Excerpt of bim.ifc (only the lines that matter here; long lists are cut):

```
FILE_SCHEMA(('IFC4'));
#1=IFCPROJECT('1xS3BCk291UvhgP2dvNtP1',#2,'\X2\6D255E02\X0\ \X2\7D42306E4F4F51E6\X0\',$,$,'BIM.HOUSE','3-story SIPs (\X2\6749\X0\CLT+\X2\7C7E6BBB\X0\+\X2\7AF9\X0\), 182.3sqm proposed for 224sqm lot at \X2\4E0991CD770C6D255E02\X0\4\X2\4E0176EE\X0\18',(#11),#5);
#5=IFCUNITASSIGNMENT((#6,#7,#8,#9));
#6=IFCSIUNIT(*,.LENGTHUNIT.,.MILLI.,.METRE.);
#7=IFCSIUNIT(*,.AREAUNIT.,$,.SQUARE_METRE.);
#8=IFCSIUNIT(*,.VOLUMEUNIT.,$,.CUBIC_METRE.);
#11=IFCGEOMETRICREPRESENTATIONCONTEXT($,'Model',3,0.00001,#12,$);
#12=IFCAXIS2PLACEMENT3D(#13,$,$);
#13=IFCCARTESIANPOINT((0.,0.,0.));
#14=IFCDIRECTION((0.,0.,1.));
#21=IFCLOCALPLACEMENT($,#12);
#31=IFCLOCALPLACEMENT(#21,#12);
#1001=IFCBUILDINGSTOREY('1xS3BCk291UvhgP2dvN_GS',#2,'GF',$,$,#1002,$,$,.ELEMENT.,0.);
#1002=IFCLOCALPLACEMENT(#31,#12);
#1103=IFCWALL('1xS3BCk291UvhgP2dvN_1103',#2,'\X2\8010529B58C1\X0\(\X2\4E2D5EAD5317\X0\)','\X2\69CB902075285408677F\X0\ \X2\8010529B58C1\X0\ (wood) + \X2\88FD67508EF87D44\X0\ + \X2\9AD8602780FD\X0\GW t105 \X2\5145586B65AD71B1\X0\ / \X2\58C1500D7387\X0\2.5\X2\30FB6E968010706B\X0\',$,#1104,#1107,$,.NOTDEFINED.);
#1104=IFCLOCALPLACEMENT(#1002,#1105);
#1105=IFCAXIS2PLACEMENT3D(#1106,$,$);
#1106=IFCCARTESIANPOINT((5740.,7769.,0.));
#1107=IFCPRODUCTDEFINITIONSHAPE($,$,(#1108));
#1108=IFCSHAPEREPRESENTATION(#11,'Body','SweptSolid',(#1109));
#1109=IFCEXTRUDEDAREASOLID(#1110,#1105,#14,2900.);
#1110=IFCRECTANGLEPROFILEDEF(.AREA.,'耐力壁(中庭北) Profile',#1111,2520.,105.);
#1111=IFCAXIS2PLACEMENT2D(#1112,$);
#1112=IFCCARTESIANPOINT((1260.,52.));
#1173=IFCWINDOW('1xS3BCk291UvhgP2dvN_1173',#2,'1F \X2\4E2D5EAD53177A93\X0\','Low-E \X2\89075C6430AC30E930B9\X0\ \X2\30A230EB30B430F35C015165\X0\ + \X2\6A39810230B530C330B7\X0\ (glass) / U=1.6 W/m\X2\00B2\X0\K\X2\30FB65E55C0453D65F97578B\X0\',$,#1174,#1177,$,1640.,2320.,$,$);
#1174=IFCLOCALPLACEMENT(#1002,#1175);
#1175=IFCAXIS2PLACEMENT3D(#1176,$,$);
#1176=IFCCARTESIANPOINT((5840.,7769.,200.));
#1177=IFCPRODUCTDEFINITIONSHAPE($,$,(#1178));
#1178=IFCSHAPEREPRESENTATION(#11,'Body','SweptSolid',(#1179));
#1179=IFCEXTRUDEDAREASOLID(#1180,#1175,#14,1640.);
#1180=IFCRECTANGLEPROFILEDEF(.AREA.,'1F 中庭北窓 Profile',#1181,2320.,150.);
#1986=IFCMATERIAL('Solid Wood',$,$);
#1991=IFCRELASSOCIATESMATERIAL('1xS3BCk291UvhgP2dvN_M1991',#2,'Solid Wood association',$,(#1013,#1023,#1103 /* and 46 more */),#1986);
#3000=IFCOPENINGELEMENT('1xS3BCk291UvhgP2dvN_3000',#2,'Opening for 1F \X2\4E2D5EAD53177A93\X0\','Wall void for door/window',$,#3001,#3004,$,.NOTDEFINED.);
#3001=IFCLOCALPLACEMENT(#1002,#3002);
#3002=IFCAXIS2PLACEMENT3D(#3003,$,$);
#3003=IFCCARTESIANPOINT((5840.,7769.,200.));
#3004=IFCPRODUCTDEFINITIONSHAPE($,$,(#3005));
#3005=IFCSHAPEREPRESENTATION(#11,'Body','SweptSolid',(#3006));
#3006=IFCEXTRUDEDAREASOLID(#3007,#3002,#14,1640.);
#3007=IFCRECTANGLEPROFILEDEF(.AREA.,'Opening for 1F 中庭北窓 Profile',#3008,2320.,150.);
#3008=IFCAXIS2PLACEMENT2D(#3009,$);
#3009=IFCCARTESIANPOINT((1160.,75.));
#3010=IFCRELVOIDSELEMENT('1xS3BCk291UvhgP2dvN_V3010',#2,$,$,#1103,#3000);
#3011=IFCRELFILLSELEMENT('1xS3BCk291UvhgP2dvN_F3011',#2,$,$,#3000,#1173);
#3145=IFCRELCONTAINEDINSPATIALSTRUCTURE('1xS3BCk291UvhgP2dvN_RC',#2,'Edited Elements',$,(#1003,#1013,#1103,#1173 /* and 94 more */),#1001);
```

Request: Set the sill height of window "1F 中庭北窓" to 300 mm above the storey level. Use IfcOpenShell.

```python
import numpy as np
import ifcopenshell
import ifcopenshell.api.geometry
import ifcopenshell.geom
import ifcopenshell.util.element
import ifcopenshell.util.placement
import ifcopenshell.util.shape
import ifcopenshell.util.unit

model = ifcopenshell.open("bim.ifc")
unit_scale = ifcopenshell.util.unit.calculate_unit_scale(model)

window = model.by_guid("1xS3BCk291UvhgP2dvN_1173")
opening = window.FillsVoids[0].RelatingOpeningElement
storey = ifcopenshell.util.element.get_container(window, ifc_class="IfcBuildingStorey")
level = ifcopenshell.util.placement.get_local_placement(storey.ObjectPlacement)[2, 3]

# The opening's origin need not be at the sill, so measure its lowest point.
shape = ifcopenshell.geom.create_shape(ifcopenshell.geom.settings(), opening)
bottom = ifcopenshell.util.shape.get_shape_bottom_elevation(shape, shape.geometry) / unit_scale
dz = level + 300.0 - bottom

shift = np.array([0.0, 0.0, dz])
# The window is not placed relative to its opening, so move both.
for product in (opening, window):
    matrix = ifcopenshell.util.placement.get_local_placement(product.ObjectPlacement)
    matrix[:3, 3] += shift
    ifcopenshell.api.geometry.edit_object_placement(model, product=product, matrix=matrix, is_si=False)

print(f"moved by {dz * unit_scale:+.3f} m")

model.write("bim-out.ifc")
```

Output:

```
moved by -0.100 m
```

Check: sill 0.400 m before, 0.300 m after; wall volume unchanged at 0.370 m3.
